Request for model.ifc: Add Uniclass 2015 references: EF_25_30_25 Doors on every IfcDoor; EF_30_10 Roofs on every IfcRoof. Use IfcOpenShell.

First a look at what the model holds.

```python
import ifcopenshell

model = ifcopenshell.open("model.ifc")
print(model.schema)
print("classifications:", [c.Name for c in model.by_type("IfcClassification")])
for ifc_class in ("IfcDoor", "IfcRoof", "IfcStair", "IfcWall", "IfcWindow"):
    print(ifc_class, len(model.by_type(ifc_class)))
```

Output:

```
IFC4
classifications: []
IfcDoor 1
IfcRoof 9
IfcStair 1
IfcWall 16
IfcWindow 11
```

```python
import ifcopenshell
import ifcopenshell.api.classification

model = ifcopenshell.open("model.ifc")

system = ifcopenshell.api.classification.add_classification(model, classification="Uniclass 2015")

codes = {
    "IfcDoor": ("EF_25_30_25", "Doors"),
    "IfcRoof": ("EF_30_10", "Roofs"),
}
for ifc_class, (code, name) in codes.items():
    products = model.by_type(ifc_class)
    ifcopenshell.api.classification.add_reference(
        model, products=products, classification=system, identification=code, name=name
    )
    print(code, len(products))

model.write("model_edited.ifc")
```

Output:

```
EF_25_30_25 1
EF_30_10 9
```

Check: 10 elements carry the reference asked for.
